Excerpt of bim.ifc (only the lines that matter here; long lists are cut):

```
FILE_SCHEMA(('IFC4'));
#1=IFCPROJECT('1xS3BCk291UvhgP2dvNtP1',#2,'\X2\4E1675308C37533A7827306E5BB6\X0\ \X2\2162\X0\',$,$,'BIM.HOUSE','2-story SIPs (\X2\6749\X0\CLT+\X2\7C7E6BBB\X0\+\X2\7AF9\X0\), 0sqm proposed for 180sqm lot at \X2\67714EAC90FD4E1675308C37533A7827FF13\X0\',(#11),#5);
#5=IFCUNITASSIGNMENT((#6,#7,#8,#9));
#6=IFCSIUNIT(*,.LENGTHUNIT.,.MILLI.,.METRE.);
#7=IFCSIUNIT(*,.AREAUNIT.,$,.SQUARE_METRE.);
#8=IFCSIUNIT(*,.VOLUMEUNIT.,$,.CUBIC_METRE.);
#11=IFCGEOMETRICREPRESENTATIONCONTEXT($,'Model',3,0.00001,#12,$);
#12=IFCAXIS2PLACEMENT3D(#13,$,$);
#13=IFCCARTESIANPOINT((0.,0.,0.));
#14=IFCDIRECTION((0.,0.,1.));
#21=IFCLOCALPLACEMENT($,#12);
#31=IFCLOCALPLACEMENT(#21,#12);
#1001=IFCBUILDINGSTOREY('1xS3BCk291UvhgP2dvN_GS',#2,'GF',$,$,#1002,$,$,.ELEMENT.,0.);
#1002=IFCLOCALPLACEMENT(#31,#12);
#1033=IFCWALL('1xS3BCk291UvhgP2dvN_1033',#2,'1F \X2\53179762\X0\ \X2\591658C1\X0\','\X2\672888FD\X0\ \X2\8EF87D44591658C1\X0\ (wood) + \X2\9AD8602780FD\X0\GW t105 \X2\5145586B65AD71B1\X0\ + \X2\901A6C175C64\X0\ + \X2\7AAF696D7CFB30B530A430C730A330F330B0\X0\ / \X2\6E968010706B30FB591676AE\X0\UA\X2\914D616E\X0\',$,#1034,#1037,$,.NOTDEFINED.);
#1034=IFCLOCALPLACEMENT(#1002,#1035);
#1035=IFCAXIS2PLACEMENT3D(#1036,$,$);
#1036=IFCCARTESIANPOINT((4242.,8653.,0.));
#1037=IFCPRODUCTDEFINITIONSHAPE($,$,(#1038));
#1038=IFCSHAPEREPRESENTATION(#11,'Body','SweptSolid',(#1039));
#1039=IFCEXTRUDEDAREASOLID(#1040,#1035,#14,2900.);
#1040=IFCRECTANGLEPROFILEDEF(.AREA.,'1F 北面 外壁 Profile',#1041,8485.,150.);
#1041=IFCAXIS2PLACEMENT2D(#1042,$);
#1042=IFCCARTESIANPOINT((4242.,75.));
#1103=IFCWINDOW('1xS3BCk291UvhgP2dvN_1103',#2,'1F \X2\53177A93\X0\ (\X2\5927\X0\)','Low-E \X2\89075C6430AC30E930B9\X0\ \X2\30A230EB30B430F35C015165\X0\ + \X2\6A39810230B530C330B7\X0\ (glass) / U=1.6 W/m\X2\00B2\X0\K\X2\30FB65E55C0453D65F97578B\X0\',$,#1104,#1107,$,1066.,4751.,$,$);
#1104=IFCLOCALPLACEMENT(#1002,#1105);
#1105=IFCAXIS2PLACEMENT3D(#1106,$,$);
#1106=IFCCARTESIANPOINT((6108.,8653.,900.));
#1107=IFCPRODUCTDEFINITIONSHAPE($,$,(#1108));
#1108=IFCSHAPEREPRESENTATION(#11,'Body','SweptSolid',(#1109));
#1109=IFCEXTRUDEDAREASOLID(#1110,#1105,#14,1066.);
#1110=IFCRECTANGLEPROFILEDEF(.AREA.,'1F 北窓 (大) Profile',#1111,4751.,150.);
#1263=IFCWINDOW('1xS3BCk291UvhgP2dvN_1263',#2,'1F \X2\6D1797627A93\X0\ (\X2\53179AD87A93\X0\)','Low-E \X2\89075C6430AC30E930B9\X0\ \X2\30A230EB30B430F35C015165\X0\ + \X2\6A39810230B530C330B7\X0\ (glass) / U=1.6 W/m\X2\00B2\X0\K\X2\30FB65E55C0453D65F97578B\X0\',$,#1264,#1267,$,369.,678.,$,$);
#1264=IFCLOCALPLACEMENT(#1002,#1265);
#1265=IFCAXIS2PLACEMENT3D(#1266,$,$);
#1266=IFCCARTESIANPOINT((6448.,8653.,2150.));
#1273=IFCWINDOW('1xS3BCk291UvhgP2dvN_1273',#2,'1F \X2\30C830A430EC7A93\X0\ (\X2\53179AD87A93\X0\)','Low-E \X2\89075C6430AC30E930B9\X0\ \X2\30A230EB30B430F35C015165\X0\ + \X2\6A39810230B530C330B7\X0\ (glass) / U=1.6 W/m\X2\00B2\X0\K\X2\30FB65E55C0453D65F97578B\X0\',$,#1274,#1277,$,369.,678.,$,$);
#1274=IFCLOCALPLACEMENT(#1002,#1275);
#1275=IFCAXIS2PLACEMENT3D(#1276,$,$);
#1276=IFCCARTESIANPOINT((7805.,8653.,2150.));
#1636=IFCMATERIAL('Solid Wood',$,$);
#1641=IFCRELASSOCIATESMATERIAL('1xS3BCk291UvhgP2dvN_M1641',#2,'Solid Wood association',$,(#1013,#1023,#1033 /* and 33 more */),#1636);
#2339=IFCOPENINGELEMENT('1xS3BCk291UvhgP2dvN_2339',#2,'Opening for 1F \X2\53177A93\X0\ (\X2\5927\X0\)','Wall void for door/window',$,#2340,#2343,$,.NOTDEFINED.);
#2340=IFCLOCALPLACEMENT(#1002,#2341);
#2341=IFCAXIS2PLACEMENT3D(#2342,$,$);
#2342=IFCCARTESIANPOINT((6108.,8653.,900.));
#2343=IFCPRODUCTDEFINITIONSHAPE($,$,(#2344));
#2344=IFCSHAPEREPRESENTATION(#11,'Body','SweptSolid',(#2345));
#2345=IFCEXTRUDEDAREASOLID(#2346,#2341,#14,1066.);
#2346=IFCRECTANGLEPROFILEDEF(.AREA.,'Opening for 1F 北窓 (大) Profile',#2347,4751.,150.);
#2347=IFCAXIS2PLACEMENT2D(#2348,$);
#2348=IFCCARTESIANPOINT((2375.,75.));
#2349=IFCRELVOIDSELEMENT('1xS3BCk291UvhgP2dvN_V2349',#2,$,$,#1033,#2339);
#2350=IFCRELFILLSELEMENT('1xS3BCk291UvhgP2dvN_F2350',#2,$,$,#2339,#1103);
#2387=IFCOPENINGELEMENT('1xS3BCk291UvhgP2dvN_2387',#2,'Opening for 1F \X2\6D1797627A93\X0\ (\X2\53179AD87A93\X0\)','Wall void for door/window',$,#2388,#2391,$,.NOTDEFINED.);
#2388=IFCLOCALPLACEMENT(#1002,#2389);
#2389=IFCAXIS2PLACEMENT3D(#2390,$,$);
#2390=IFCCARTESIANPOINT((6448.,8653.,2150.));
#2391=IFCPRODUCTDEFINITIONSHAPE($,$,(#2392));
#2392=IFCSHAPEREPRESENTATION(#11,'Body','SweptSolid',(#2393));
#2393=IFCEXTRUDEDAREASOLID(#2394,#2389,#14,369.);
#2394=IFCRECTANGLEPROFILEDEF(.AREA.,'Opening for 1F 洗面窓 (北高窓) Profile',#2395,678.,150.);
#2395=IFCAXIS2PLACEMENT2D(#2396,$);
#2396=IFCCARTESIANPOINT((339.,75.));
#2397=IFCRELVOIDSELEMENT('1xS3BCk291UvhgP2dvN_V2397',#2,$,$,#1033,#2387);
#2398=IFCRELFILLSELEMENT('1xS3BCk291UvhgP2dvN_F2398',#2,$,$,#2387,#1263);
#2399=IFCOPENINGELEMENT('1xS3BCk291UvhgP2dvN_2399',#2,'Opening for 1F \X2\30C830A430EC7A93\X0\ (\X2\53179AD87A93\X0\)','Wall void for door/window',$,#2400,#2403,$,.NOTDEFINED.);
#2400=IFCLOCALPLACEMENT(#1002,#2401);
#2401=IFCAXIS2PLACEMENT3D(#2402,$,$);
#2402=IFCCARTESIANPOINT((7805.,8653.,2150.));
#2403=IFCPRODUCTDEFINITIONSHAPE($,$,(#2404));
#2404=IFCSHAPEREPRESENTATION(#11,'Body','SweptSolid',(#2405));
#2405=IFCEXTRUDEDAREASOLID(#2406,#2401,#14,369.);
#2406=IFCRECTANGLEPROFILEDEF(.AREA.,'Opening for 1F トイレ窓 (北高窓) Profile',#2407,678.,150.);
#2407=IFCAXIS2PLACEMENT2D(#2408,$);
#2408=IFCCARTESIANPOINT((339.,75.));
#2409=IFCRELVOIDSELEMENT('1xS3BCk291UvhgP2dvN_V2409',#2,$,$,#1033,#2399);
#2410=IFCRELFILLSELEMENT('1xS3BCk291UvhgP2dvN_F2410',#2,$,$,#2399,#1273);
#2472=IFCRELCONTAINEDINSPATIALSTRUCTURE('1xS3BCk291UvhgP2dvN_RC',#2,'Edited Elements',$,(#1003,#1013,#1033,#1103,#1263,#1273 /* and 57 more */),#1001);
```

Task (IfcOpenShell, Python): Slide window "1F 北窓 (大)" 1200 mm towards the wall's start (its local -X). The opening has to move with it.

```python
import ifcopenshell
import ifcopenshell.api.geometry
import ifcopenshell.util.placement
import ifcopenshell.util.unit

model = ifcopenshell.open("bim.ifc")
unit_scale = ifcopenshell.util.unit.calculate_unit_scale(model)

window = model.by_guid("1xS3BCk291UvhgP2dvN_1103")
opening = window.FillsVoids[0].RelatingOpeningElement
wall = opening.VoidsElements[0].RelatingBuildingElement

wall_matrix = ifcopenshell.util.placement.get_local_placement(wall.ObjectPlacement)
shift = wall_matrix[:3, 0] * -1.2 / unit_scale
before = ifcopenshell.util.placement.get_local_placement(window.ObjectPlacement)[:3, 3].copy()

# The window is not placed relative to its opening, so move both.
for product in (opening, window):
    matrix = ifcopenshell.util.placement.get_local_placement(product.ObjectPlacement)
    matrix[:3, 3] += shift
    ifcopenshell.api.geometry.edit_object_placement(model, product=product, matrix=matrix, is_si=False)

after = ifcopenshell.util.placement.get_local_placement(window.ObjectPlacement)[:3, 3]
print("window moved by", (after - before).round(3) + 0.0)

model.write("bim_updated.ifc")
```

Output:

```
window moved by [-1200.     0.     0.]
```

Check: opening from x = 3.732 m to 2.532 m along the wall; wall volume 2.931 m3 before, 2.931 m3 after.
